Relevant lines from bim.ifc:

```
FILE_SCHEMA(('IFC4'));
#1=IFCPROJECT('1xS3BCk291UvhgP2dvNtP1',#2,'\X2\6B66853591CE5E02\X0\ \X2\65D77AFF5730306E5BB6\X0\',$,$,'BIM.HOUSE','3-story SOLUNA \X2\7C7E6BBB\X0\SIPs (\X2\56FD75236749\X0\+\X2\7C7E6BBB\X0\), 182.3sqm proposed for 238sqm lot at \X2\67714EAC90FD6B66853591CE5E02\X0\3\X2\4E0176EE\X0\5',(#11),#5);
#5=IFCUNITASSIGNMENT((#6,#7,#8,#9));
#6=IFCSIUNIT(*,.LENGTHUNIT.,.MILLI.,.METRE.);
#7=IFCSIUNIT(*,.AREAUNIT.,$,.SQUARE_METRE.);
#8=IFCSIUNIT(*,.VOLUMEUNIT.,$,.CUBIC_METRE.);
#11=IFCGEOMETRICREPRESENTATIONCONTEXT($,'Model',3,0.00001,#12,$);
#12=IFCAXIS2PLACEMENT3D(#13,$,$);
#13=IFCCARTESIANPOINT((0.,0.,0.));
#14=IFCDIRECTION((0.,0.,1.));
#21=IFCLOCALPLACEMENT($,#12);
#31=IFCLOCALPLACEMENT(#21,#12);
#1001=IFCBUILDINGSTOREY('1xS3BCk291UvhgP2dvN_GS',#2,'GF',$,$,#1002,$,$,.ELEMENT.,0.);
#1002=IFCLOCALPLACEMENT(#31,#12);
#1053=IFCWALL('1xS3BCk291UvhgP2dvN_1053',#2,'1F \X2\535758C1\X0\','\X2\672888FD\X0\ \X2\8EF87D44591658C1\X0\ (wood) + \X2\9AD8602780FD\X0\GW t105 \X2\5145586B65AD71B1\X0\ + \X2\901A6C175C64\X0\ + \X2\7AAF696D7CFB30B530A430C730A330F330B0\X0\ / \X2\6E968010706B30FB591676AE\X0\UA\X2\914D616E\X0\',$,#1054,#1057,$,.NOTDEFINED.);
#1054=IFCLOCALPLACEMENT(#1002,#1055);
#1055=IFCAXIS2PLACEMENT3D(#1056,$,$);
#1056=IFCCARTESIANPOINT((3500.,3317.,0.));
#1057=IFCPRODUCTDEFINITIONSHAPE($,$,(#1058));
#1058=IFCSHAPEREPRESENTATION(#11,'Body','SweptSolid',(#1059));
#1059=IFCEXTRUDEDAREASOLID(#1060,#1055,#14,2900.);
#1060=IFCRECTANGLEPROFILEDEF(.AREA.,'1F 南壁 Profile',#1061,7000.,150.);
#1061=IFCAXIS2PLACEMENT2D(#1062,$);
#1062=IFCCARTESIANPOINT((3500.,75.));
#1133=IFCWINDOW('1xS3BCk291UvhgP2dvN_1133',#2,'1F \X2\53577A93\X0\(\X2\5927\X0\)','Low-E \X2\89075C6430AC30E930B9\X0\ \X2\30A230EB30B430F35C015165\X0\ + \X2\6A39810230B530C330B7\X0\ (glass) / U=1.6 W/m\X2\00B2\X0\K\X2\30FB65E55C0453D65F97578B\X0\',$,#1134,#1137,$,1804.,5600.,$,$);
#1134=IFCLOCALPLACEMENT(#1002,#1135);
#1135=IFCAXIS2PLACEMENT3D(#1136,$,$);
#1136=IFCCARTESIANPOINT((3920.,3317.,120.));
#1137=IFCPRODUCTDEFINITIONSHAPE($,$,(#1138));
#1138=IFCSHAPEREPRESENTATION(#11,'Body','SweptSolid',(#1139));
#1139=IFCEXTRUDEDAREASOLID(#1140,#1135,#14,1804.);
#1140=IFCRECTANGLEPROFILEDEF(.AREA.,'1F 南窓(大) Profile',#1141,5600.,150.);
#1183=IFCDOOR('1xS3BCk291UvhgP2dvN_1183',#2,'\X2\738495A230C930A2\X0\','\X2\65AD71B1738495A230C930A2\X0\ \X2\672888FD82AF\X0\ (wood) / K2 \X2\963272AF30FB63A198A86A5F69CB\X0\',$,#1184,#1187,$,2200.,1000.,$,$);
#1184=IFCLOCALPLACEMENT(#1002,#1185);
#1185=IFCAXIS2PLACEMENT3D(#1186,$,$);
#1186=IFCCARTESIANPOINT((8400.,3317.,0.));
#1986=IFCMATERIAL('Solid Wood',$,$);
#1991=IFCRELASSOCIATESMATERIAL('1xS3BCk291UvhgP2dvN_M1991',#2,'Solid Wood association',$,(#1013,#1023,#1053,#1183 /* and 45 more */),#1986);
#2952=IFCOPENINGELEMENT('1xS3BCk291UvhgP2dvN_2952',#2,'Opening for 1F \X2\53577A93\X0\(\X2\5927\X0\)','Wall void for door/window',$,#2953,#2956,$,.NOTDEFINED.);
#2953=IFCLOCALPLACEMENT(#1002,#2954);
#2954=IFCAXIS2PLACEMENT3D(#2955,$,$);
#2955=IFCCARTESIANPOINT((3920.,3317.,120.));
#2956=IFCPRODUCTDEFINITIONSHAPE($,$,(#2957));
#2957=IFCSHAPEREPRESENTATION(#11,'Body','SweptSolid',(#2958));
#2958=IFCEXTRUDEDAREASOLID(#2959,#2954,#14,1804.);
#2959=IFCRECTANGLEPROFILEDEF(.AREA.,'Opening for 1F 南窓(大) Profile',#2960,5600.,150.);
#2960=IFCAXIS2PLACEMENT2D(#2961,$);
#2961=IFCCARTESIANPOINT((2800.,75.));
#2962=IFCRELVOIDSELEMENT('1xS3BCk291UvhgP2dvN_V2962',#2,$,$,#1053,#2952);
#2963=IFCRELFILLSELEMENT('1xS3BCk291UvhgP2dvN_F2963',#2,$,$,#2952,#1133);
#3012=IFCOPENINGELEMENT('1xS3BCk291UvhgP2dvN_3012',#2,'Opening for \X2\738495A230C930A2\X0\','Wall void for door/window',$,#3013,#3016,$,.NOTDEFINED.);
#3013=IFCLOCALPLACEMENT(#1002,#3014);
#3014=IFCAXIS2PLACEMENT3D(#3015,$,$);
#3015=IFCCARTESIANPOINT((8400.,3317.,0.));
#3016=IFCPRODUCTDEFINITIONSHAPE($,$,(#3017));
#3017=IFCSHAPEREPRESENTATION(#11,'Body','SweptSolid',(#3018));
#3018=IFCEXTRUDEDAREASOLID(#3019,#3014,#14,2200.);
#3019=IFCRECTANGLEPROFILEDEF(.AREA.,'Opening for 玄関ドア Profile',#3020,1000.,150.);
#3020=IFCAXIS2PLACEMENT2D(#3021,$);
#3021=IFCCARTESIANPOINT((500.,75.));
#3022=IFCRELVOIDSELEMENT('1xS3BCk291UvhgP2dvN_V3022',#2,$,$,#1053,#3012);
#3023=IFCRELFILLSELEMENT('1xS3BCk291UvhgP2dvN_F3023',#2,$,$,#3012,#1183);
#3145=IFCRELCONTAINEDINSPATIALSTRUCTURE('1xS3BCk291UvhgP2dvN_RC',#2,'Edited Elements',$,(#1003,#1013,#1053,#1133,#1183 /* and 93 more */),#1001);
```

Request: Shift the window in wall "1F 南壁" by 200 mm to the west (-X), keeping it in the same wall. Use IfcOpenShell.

```python
import ifcopenshell
import ifcopenshell.api.geometry
import ifcopenshell.util.placement
import ifcopenshell.util.unit

model = ifcopenshell.open("bim.ifc")
unit_scale = ifcopenshell.util.unit.calculate_unit_scale(model)

window = model.by_guid("1xS3BCk291UvhgP2dvN_1133")
opening = window.FillsVoids[0].RelatingOpeningElement
wall = opening.VoidsElements[0].RelatingBuildingElement

wall_matrix = ifcopenshell.util.placement.get_local_placement(wall.ObjectPlacement)
shift = wall_matrix[:3, 0] * -0.2 / unit_scale
before = ifcopenshell.util.placement.get_local_placement(window.ObjectPlacement)[:3, 3].copy()

# The window is not placed relative to its opening, so move both.
for product in (opening, window):
    matrix = ifcopenshell.util.placement.get_local_placement(product.ObjectPlacement)
    matrix[:3, 3] += shift
    ifcopenshell.api.geometry.edit_object_placement(model, product=product, matrix=matrix, is_si=False)

after = ifcopenshell.util.placement.get_local_placement(window.ObjectPlacement)[:3, 3]
print("window moved by", (after - before).round(3) + 0.0)

model.write("bim_edited.ifc")
```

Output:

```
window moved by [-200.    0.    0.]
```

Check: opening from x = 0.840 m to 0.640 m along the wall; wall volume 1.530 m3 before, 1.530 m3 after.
